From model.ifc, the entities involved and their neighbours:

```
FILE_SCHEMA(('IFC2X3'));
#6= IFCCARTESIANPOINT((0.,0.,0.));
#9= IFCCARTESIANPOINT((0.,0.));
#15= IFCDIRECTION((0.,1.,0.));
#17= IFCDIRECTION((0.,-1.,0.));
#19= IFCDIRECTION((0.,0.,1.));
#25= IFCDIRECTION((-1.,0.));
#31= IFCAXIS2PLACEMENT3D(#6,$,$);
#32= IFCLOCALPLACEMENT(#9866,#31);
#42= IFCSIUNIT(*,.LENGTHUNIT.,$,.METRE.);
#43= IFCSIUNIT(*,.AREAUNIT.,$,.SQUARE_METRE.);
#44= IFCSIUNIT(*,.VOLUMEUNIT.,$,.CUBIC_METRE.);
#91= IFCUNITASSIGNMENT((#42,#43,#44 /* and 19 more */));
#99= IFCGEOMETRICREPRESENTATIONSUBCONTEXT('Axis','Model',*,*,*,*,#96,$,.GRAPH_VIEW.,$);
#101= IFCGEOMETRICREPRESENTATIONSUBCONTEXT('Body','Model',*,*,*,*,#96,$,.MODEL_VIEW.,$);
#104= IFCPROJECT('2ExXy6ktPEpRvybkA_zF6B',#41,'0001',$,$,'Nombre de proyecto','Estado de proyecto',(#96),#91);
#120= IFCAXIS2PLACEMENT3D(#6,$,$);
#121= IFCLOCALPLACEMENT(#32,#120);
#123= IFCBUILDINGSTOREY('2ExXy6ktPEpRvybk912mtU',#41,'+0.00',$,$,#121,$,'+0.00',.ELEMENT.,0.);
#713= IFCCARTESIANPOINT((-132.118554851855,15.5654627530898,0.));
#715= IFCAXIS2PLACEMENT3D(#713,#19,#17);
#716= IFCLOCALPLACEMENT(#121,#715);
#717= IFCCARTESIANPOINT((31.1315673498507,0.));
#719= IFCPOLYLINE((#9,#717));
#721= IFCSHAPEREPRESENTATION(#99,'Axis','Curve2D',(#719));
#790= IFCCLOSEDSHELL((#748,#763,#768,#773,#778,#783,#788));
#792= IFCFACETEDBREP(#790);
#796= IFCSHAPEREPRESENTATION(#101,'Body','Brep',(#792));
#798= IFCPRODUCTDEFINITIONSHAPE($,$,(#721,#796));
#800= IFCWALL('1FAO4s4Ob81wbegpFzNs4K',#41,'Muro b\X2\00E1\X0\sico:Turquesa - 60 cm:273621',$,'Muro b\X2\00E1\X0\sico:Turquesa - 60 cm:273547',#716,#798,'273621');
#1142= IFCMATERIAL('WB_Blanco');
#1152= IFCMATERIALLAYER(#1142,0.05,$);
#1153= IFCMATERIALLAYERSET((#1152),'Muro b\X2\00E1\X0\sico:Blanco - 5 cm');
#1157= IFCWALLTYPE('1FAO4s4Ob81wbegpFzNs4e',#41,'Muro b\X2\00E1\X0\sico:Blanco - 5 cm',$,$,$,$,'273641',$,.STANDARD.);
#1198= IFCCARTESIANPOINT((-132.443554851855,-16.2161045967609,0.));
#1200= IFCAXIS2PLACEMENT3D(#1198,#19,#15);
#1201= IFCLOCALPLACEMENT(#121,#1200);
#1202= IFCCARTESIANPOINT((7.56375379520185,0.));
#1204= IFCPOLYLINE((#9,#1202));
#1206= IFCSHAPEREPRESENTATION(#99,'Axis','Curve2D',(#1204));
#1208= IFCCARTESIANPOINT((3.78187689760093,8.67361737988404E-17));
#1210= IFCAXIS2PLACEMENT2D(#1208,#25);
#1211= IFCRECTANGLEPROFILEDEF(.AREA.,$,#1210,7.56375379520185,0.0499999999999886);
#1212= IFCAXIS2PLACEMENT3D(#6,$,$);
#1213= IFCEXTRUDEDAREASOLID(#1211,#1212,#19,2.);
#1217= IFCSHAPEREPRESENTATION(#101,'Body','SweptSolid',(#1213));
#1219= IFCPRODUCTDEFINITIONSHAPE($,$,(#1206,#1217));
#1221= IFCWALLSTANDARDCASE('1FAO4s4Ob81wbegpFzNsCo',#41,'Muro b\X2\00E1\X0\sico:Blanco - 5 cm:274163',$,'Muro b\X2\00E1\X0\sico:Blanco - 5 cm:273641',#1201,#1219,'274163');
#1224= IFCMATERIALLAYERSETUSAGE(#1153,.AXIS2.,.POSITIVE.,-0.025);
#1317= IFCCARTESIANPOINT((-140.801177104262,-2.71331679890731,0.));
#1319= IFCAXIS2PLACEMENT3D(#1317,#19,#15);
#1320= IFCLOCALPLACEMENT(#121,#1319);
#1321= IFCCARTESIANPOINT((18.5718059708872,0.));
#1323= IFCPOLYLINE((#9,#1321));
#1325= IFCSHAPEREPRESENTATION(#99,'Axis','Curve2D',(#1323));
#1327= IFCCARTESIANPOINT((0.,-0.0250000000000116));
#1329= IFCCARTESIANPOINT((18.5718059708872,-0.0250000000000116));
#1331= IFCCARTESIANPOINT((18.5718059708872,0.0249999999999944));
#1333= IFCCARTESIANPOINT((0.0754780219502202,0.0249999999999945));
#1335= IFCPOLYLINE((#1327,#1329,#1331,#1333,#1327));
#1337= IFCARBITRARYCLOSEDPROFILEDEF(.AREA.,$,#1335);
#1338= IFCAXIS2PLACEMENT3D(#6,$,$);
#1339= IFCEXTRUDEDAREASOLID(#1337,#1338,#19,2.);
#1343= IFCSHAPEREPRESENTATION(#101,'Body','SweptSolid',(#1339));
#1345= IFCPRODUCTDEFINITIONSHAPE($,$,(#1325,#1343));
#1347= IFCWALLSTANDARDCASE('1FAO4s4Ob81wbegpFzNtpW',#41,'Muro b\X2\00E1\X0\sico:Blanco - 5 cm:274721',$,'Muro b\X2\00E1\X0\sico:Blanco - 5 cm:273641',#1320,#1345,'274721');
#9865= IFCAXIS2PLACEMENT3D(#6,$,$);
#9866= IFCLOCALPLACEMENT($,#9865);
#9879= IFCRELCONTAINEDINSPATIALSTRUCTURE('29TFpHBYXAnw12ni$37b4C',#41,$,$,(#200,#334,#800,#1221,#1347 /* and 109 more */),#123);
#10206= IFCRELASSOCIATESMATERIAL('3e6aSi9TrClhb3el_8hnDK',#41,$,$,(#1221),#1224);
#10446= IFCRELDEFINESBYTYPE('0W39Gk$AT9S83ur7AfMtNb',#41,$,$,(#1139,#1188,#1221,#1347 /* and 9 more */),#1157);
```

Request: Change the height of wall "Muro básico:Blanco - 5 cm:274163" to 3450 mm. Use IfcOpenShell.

```python
import ifcopenshell
import ifcopenshell.geom
import ifcopenshell.util.representation
import ifcopenshell.util.shape

model = ifcopenshell.open("model.ifc")
settings = ifcopenshell.geom.settings()


def volume(element):
    """Net volume in cubic metres, openings subtracted."""
    shape = ifcopenshell.geom.create_shape(settings, element)
    return ifcopenshell.util.shape.get_volume(shape.geometry)


wall = model.by_guid("1FAO4s4Ob81wbegpFzNsCo")
before = volume(wall)

body = ifcopenshell.util.representation.get_representation(wall, "Model", "Body")
solid = body.Items[0]
old_height = solid.Depth
solid.Depth = 3.45
after = volume(wall)

print(f"height {old_height:g} -> {solid.Depth:g}, volume {before:.3f} -> {after:.3f} m3")

model.write("model-out.ifc")
```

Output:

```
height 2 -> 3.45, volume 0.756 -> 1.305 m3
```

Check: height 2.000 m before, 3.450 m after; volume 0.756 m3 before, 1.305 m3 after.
